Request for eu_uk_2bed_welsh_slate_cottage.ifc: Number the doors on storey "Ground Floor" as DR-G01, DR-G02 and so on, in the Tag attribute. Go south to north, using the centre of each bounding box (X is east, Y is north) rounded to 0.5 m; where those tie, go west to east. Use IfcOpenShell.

First a look at what the model holds.

```python
import ifcopenshell
import ifcopenshell.util.element
import ifcopenshell.util.placement

model = ifcopenshell.open("eu_uk_2bed_welsh_slate_cottage.ifc")
print(model.schema)
storey = next(s for s in model.by_type("IfcBuildingStorey") if s.Name == "Ground Floor")
doors = [e for e in ifcopenshell.util.element.get_decomposition(storey) if e.is_a("IfcDoor")]
for e in sorted(doors, key=lambda e: e.id()):
    origin = ifcopenshell.util.placement.get_local_placement(e.ObjectPlacement)[:3, 3]
    print(e.id(), e.Tag, e.Name, origin.round(2) + 0.0, sep=" | ")
```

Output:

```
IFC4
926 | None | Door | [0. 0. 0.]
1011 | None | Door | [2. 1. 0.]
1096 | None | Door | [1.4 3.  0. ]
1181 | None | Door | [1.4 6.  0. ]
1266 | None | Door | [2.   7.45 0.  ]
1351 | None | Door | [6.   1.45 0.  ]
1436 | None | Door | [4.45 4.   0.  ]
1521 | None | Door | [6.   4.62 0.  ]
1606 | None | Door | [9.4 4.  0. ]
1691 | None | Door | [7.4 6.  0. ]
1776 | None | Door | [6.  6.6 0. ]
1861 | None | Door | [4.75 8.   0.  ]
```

```python
import ifcopenshell
import ifcopenshell.geom
import ifcopenshell.util.element
import ifcopenshell.util.shape

model = ifcopenshell.open("eu_uk_2bed_welsh_slate_cottage.ifc")
settings = ifcopenshell.geom.settings()
settings.set("use-world-coords", True)


def centre(element):
    shape = ifcopenshell.geom.create_shape(settings, element)
    return ifcopenshell.util.shape.get_bbox_centroid(shape.geometry)


storey = next(s for s in model.by_type("IfcBuildingStorey") if s.Name == "Ground Floor")
doors = [e for e in ifcopenshell.util.element.get_decomposition(storey) if e.is_a("IfcDoor")]

# Insertion points can sit at a corner or the storey origin, so sort by the geometry (in metres).
centres = {e: centre(e) for e in doors}
doors.sort(key=lambda e: (round(centres[e][1] / 0.5), centres[e][0]))

for i, e in enumerate(doors, start=1):
    number = f"DR-G{i:02d}"
    e.Tag = number
    print(e.id(), number)

model.write("eu_uk_2bed_welsh_slate_cottage_updated.ifc")
```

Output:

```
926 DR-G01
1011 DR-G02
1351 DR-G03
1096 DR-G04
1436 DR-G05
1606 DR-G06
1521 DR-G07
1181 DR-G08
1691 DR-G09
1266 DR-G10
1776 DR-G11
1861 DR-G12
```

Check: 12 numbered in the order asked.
